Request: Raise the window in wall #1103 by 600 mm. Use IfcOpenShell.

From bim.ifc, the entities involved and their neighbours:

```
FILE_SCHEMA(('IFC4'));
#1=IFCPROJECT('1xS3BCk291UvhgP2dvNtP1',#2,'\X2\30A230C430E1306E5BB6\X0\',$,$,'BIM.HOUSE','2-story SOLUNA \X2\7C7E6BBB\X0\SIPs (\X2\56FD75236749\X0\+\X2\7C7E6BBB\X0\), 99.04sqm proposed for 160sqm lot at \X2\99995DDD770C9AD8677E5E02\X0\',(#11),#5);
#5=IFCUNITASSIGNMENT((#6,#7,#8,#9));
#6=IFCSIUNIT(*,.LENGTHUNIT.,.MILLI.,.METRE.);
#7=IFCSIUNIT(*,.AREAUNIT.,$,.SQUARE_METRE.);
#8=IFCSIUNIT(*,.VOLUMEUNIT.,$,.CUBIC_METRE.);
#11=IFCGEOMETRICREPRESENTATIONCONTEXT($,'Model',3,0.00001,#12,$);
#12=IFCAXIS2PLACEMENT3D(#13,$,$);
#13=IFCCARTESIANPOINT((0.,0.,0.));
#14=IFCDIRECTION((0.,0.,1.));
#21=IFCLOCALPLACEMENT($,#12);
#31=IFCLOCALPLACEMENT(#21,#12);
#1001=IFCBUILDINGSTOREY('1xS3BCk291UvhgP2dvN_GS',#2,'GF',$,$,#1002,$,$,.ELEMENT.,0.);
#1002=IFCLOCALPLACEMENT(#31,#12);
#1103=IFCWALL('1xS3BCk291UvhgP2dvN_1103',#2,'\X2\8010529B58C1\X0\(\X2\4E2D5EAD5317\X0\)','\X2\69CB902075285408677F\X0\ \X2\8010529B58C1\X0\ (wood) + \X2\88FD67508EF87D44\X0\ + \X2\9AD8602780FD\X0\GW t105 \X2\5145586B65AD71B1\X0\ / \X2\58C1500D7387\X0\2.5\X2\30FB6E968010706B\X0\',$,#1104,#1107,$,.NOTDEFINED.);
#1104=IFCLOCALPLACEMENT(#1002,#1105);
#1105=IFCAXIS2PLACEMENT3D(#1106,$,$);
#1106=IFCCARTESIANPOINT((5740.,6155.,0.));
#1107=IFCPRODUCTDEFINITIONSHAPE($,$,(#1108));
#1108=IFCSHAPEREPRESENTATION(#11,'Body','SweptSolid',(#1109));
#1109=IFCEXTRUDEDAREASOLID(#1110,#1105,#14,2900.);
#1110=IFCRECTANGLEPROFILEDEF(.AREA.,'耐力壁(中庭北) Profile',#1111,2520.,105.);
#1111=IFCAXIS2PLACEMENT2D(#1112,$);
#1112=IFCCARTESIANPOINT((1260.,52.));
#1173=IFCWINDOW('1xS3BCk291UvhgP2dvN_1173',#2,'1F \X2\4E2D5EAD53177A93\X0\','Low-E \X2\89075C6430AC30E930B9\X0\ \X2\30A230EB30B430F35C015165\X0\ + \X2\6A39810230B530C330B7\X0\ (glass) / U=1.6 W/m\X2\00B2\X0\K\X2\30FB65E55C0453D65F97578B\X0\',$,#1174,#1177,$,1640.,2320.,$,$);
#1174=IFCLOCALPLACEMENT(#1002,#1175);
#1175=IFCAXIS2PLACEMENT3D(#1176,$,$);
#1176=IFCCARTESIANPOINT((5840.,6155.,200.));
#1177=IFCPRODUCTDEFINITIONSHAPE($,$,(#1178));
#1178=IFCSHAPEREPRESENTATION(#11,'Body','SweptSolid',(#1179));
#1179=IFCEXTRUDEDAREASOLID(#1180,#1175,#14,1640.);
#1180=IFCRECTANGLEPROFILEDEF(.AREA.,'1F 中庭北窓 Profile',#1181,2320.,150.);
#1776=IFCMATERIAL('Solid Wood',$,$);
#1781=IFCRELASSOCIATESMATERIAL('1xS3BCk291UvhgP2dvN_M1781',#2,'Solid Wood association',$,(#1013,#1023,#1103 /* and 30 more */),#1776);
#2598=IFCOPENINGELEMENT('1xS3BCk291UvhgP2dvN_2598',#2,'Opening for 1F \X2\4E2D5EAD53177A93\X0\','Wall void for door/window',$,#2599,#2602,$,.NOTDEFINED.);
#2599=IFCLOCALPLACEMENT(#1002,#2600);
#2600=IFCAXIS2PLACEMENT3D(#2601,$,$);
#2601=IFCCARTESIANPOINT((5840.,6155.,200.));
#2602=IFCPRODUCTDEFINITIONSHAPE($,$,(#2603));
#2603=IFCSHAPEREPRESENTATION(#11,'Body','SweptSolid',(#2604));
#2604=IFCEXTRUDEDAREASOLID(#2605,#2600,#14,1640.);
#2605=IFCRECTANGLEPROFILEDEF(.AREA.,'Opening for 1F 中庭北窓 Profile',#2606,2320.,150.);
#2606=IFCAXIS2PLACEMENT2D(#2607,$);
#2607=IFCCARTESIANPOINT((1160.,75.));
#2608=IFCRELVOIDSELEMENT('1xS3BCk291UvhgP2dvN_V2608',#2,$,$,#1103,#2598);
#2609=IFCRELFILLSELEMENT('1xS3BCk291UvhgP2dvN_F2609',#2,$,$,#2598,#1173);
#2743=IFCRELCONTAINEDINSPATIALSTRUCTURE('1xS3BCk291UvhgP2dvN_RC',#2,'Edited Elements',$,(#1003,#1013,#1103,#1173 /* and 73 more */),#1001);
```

```python
import numpy as np
import ifcopenshell
import ifcopenshell.api.geometry
import ifcopenshell.util.placement
import ifcopenshell.util.unit

model = ifcopenshell.open("bim.ifc")
unit_scale = ifcopenshell.util.unit.calculate_unit_scale(model)

window = model.by_guid("1xS3BCk291UvhgP2dvN_1173")
opening = window.FillsVoids[0].RelatingOpeningElement
dz = 0.6 / unit_scale

shift = np.array([0.0, 0.0, dz])
# The window is not placed relative to its opening, so move both.
for product in (opening, window):
    matrix = ifcopenshell.util.placement.get_local_placement(product.ObjectPlacement)
    matrix[:3, 3] += shift
    ifcopenshell.api.geometry.edit_object_placement(model, product=product, matrix=matrix, is_si=False)

print(f"moved by {dz * unit_scale:+.3f} m")

model.write("bim_v2.ifc")
```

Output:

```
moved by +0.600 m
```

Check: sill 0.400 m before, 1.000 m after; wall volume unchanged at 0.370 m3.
